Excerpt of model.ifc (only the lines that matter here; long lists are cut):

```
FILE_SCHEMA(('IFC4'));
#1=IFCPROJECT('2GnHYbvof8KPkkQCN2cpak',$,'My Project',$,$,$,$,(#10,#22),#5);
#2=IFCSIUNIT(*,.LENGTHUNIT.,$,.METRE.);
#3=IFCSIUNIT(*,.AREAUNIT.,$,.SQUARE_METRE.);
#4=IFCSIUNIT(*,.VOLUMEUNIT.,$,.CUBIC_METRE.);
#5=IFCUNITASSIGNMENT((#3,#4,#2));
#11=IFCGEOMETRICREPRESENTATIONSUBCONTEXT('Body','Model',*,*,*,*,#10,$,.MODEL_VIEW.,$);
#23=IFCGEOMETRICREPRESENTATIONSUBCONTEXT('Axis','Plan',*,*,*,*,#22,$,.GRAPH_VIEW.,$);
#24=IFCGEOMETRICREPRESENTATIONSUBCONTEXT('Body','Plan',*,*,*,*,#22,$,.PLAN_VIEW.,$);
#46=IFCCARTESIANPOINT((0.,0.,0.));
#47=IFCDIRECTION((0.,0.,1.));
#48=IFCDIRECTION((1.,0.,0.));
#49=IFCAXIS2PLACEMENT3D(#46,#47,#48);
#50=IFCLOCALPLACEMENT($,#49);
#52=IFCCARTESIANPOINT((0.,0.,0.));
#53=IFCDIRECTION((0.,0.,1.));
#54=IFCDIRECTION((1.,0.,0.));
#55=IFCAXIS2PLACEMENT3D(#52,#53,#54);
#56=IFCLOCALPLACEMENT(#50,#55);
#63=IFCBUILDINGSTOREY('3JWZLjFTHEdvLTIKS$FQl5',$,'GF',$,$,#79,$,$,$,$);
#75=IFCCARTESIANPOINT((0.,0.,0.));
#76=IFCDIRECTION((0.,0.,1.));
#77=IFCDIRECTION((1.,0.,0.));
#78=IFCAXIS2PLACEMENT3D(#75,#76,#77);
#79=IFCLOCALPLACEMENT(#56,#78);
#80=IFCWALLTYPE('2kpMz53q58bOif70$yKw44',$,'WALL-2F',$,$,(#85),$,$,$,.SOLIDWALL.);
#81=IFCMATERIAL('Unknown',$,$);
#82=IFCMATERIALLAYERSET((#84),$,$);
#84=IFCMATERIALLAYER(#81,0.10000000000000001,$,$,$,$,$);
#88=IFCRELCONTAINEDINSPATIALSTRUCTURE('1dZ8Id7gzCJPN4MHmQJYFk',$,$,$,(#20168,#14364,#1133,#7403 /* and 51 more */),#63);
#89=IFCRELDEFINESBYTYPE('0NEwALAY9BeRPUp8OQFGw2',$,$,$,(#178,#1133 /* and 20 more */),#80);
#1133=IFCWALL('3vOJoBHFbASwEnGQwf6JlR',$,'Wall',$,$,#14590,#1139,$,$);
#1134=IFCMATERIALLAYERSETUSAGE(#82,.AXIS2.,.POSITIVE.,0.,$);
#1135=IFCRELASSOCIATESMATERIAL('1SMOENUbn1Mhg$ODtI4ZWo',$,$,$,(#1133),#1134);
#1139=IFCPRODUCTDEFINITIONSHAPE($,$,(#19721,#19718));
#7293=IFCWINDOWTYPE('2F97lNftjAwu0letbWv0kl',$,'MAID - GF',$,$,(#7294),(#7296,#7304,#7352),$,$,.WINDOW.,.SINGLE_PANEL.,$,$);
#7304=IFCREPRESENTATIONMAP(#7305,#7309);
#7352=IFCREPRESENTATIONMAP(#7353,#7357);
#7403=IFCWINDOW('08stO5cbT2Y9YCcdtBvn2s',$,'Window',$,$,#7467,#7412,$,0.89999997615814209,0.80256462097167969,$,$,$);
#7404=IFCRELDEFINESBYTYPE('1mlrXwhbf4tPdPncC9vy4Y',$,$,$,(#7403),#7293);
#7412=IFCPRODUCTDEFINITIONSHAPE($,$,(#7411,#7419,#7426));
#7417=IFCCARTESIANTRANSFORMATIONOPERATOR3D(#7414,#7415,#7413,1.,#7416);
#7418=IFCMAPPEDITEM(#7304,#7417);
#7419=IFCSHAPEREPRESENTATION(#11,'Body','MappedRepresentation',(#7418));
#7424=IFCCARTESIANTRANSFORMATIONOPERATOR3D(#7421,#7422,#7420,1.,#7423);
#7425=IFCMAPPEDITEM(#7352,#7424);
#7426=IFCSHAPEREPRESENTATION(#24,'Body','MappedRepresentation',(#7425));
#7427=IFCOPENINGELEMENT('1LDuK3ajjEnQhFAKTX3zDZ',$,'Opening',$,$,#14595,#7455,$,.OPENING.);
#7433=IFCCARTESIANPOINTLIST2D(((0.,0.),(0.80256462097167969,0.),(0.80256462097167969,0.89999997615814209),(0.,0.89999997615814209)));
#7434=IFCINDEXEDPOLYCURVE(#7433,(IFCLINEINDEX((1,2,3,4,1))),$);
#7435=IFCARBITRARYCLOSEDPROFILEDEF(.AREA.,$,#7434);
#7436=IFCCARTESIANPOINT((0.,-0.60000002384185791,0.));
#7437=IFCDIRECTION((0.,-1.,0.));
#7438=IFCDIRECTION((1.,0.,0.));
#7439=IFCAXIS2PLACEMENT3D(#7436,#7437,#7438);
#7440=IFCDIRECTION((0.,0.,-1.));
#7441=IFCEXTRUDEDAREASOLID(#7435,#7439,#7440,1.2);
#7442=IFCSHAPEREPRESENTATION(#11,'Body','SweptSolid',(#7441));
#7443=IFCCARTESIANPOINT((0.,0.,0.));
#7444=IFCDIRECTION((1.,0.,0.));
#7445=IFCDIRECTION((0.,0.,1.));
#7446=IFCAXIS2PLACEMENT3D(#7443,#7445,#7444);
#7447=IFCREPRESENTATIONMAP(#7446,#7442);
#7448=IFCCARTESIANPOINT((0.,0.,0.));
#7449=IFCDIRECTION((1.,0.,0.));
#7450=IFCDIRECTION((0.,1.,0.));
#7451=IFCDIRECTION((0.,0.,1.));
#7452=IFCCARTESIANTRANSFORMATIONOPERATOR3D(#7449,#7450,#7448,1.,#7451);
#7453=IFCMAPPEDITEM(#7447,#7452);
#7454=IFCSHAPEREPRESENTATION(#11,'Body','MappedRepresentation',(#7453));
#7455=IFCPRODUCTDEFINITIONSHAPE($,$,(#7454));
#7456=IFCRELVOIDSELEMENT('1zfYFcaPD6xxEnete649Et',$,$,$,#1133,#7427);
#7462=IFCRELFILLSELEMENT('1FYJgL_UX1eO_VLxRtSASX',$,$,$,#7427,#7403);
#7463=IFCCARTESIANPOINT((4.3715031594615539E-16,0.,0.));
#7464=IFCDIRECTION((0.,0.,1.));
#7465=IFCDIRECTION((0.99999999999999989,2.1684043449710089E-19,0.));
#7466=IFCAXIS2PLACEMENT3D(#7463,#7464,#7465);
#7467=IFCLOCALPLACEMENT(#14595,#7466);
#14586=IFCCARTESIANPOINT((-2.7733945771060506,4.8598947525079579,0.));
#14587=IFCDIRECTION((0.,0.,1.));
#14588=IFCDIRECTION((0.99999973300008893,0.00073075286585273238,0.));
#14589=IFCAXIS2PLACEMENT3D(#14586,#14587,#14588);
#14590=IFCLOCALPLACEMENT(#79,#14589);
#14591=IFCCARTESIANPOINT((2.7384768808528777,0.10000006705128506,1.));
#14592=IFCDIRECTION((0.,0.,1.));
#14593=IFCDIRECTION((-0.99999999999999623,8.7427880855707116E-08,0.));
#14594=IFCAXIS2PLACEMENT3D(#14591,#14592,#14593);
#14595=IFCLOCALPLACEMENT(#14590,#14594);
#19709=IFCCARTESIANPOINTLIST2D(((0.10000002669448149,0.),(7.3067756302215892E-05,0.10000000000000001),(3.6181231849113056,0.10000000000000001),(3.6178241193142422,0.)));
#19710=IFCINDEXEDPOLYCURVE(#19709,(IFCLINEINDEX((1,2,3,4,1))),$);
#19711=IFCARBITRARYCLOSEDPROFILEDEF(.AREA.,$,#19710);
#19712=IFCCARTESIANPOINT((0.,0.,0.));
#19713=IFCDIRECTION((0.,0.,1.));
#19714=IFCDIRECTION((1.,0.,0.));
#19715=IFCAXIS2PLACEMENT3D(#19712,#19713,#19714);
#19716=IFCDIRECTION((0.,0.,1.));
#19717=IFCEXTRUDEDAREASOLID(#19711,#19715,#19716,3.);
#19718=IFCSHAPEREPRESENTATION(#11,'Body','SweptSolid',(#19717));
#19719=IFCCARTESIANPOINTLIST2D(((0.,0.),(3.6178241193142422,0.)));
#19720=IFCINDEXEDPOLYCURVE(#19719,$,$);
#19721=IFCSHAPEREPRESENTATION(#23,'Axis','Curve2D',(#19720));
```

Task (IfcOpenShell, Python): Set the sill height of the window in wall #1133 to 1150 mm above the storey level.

```python
import numpy as np
import ifcopenshell
import ifcopenshell.api.geometry
import ifcopenshell.geom
import ifcopenshell.util.element
import ifcopenshell.util.placement
import ifcopenshell.util.shape
import ifcopenshell.util.unit

model = ifcopenshell.open("model.ifc")
unit_scale = ifcopenshell.util.unit.calculate_unit_scale(model)

window = model.by_guid("08stO5cbT2Y9YCcdtBvn2s")
opening = window.FillsVoids[0].RelatingOpeningElement
storey = ifcopenshell.util.element.get_container(window, ifc_class="IfcBuildingStorey")
level = ifcopenshell.util.placement.get_local_placement(storey.ObjectPlacement)[2, 3]

# The opening's origin need not be at the sill, so measure its lowest point.
shape = ifcopenshell.geom.create_shape(ifcopenshell.geom.settings(), opening)
bottom = ifcopenshell.util.shape.get_shape_bottom_elevation(shape, shape.geometry) / unit_scale
dz = level + 1.15 - bottom

shift = np.array([0.0, 0.0, dz])
# The window is placed relative to its opening, so it follows when the opening moves.
matrix = ifcopenshell.util.placement.get_local_placement(opening.ObjectPlacement)
matrix[:3, 3] += shift
ifcopenshell.api.geometry.edit_object_placement(
    model, product=opening, matrix=matrix, is_si=False, should_transform_children=True
)

print(f"moved by {dz * unit_scale:+.3f} m")

model.write("model_edited.ifc")
```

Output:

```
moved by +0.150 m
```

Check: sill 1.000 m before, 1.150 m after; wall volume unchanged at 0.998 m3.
